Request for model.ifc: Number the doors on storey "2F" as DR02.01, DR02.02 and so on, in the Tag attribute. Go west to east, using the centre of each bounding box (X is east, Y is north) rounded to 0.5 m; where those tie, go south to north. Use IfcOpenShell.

First a look at what the model holds.

```python
import ifcopenshell
import ifcopenshell.util.element
import ifcopenshell.util.placement

model = ifcopenshell.open("model.ifc")
print(model.schema)
storey = next(s for s in model.by_type("IfcBuildingStorey") if s.Name == "2F")
doors = [e for e in ifcopenshell.util.element.get_decomposition(storey) if e.is_a("IfcDoor")]
for e in sorted(doors, key=lambda e: e.id()):
    origin = ifcopenshell.util.placement.get_local_placement(e.ObjectPlacement)[:3, 3]
    print(e.id(), e.Tag, e.Name, origin.round(2) + 0.0, sep=" | ")
```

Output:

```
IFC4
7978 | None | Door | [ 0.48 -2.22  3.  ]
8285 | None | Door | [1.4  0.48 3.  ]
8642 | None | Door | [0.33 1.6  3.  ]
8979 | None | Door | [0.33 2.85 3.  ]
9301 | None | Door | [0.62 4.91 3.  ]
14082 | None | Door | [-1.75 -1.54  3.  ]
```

```python
import ifcopenshell
import ifcopenshell.geom
import ifcopenshell.util.element
import ifcopenshell.util.shape

model = ifcopenshell.open("model.ifc")
settings = ifcopenshell.geom.settings()
settings.set("use-world-coords", True)


def centre(element):
    shape = ifcopenshell.geom.create_shape(settings, element)
    return ifcopenshell.util.shape.get_bbox_centroid(shape.geometry)


storey = next(s for s in model.by_type("IfcBuildingStorey") if s.Name == "2F")
doors = [e for e in ifcopenshell.util.element.get_decomposition(storey) if e.is_a("IfcDoor")]

# Insertion points can sit at a corner or the storey origin, so sort by the geometry (in metres).
centres = {e: centre(e) for e in doors}
doors.sort(key=lambda e: (round(centres[e][0] / 0.5), centres[e][1]))

for i, e in enumerate(doors, start=1):
    number = f"DR02.{i:02d}"
    e.Tag = number
    print(e.id(), number)

model.write("model_v2.ifc")
```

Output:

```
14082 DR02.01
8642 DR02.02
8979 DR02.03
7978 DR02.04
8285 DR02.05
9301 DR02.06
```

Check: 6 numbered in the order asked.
